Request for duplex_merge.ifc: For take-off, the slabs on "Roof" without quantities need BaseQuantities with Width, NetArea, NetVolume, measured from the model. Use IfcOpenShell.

First a look at what the model holds.

```python
import ifcopenshell
import ifcopenshell.util.element
import ifcopenshell.util.unit

model = ifcopenshell.open("duplex_merge.ifc")
print(model.schema)
for unit_type in ("LENGTHUNIT", "AREAUNIT", "VOLUMEUNIT"):
    print(unit_type, ifcopenshell.util.unit.calculate_unit_scale(model, unit_type))
storey = next(s for s in model.by_type("IfcBuildingStorey") if s.Name == "Roof")
slabs = [e for e in ifcopenshell.util.element.get_decomposition(storey) if e.is_a("IfcSlab")]
for e in sorted(slabs, key=lambda e: e.id()):
    print(e.id(), e.is_a(), e.Name, list(ifcopenshell.util.element.get_psets(e, qtos_only=True)), sep=" | ")
```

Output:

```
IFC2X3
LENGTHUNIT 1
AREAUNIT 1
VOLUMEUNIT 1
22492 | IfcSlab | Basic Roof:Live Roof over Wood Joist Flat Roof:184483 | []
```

```python
import ifcopenshell
import ifcopenshell.api.pset
import ifcopenshell.geom
import ifcopenshell.util.element
import ifcopenshell.util.shape
import ifcopenshell.util.unit

model = ifcopenshell.open("duplex_merge.ifc")
unit_scale = ifcopenshell.util.unit.calculate_unit_scale(model)
area_scale = ifcopenshell.util.unit.calculate_unit_scale(model, "AREAUNIT")
volume_scale = ifcopenshell.util.unit.calculate_unit_scale(model, "VOLUMEUNIT")
settings = ifcopenshell.geom.settings()

storey = next(s for s in model.by_type("IfcBuildingStorey") if s.Name == "Roof")
slabs = [e for e in ifcopenshell.util.element.get_decomposition(storey) if e.is_a("IfcSlab")]

for e in sorted(slabs, key=lambda e: e.id()):
    if ifcopenshell.util.element.get_psets(e, qtos_only=True, should_inherit=False):
        continue
    # Geometry comes back in metres, in the element's own axes.
    shape = ifcopenshell.geom.create_shape(settings, e)
    values = {
        "Width": ifcopenshell.util.shape.get_z(shape.geometry) / unit_scale,
        "NetArea": ifcopenshell.util.shape.get_footprint_area(shape.geometry) / area_scale,
        "NetVolume": ifcopenshell.util.shape.get_volume(shape.geometry) / volume_scale,
    }
    qto = ifcopenshell.api.pset.add_qto(model, product=e, name="BaseQuantities")
    ifcopenshell.api.pset.edit_qto(model, qto=qto, properties=values)
    print(e.id(), {k: round(v, 3) for k, v in values.items()})

model.write("duplex_merge_rev.ifc")
```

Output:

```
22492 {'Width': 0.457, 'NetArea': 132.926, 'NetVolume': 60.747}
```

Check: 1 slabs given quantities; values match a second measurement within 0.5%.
